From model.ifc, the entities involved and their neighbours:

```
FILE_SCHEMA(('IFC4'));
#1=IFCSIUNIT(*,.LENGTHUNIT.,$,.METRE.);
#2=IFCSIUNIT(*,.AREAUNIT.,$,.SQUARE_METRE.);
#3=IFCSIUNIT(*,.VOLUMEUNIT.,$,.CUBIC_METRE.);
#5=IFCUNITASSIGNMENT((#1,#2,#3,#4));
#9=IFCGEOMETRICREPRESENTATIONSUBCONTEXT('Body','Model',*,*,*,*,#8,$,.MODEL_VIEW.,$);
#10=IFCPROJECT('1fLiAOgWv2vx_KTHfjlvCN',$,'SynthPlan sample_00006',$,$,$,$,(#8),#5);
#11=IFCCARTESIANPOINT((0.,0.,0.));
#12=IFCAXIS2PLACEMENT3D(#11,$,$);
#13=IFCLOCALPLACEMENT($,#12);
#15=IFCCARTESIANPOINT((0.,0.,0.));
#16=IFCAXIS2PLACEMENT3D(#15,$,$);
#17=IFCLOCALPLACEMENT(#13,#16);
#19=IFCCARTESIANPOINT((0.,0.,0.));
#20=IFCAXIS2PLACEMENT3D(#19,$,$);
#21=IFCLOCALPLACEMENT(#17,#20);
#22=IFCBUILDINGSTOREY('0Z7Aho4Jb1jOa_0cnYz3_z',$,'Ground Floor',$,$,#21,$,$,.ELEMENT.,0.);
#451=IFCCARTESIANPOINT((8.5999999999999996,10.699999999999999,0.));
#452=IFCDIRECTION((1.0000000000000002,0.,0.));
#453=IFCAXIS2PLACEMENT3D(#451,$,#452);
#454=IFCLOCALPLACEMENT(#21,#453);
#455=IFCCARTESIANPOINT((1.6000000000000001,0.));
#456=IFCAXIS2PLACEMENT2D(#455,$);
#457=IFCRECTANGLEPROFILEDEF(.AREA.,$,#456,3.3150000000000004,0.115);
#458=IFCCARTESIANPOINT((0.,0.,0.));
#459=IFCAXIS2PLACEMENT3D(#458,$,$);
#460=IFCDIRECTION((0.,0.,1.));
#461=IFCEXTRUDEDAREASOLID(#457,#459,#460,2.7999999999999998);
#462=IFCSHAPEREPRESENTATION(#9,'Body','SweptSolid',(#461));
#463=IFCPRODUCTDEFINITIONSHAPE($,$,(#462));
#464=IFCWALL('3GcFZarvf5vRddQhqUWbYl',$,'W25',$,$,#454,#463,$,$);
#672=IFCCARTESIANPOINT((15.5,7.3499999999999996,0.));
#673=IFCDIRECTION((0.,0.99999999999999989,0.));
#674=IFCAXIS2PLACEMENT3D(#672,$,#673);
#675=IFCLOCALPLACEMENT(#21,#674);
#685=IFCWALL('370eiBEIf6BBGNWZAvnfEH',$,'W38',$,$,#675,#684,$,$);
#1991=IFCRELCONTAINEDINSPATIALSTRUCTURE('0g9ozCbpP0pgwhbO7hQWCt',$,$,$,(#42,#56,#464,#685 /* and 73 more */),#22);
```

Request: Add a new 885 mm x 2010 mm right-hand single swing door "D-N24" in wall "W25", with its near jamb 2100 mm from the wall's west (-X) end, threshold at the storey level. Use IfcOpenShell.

```python
import numpy as np
import ifcopenshell
import ifcopenshell.api.feature
import ifcopenshell.api.geometry
import ifcopenshell.api.root
import ifcopenshell.api.spatial
import ifcopenshell.geom
import ifcopenshell.util.element
import ifcopenshell.util.placement
import ifcopenshell.util.representation
import ifcopenshell.util.shape
import ifcopenshell.util.unit

model = ifcopenshell.open("model.ifc")
unit_scale = ifcopenshell.util.unit.calculate_unit_scale(model)
settings = ifcopenshell.geom.settings()


def volume(element):
    """Net volume in cubic metres, openings subtracted."""
    shape = ifcopenshell.geom.create_shape(settings, element)
    return ifcopenshell.util.shape.get_volume(shape.geometry)


wall = model.by_guid("3GcFZarvf5vRddQhqUWbYl")
storey = ifcopenshell.util.element.get_container(wall, ifc_class="IfcBuildingStorey")
context = ifcopenshell.util.representation.get_context(model, "Model", "Body", "MODEL_VIEW")
before = volume(wall)

width, height, from_end, sill = 0.885, 2.01, 2.1, 0.0  # metres

# The wall runs along its own X axis, and the end named is its -X end.
wall_shape = ifcopenshell.geom.create_shape(settings, wall)
x, y, z = ifcopenshell.util.shape.get_vertices(wall_shape.geometry).T
start = x.min() + from_end
face, thickness = float(y.min()), float(y.max() - y.min())
wall_matrix = ifcopenshell.util.placement.get_local_placement(wall.ObjectPlacement)
level = ifcopenshell.util.placement.get_local_placement(storey.ObjectPlacement)[2, 3]


def in_wall(x, y):
    """Placement at x, y metres in the wall's axes, at sill height."""
    matrix = wall_matrix.copy()
    matrix[:, 3] = wall_matrix @ np.array([x / unit_scale, y / unit_scale, 0.0, 1.0])
    matrix[2, 3] = level + sill / unit_scale
    return matrix


# Opening: a box that overshoots both wall faces by 50 mm.
opening = ifcopenshell.api.root.create_entity(model, ifc_class="IfcOpeningElement", predefined_type="OPENING")
box = ifcopenshell.api.geometry.add_wall_representation(
    model, context=context, length=width, height=height, thickness=thickness + 0.1
)
ifcopenshell.api.geometry.assign_representation(model, product=opening, representation=box)
ifcopenshell.api.geometry.edit_object_placement(model, product=opening, matrix=in_wall(start, face - 0.05), is_si=False)
ifcopenshell.api.feature.add_feature(model, feature=opening, element=wall)

door = ifcopenshell.api.root.create_entity(model, ifc_class="IfcDoor", name="D-N24", predefined_type="DOOR")
door.OverallWidth, door.OverallHeight = width / unit_scale, height / unit_scale
door.OperationType = "SINGLE_SWING_RIGHT"
body = ifcopenshell.api.geometry.add_door_representation(
    model,
    context=context,
    overall_width=door.OverallWidth,
    overall_height=door.OverallHeight,
    operation_type="SINGLE_SWING_RIGHT",
    lining_properties={"LiningDepth": thickness / unit_scale, "ThresholdDepth": thickness / unit_scale},
)
ifcopenshell.api.geometry.assign_representation(model, product=door, representation=body)
ifcopenshell.api.spatial.assign_container(model, products=[door], relating_structure=storey)
ifcopenshell.api.feature.add_filling(model, opening=opening, element=door)

# The lining spans the wall, so the door starts at the wall face.
ifcopenshell.api.geometry.edit_object_placement(model, product=door, matrix=in_wall(start, face), is_si=False)

after = volume(wall)

print(f"wall volume {before:.3f} -> {after:.3f} m3")

model.write("model_updated.ifc")
```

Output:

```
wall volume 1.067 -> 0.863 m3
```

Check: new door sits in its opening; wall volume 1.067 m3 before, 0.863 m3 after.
